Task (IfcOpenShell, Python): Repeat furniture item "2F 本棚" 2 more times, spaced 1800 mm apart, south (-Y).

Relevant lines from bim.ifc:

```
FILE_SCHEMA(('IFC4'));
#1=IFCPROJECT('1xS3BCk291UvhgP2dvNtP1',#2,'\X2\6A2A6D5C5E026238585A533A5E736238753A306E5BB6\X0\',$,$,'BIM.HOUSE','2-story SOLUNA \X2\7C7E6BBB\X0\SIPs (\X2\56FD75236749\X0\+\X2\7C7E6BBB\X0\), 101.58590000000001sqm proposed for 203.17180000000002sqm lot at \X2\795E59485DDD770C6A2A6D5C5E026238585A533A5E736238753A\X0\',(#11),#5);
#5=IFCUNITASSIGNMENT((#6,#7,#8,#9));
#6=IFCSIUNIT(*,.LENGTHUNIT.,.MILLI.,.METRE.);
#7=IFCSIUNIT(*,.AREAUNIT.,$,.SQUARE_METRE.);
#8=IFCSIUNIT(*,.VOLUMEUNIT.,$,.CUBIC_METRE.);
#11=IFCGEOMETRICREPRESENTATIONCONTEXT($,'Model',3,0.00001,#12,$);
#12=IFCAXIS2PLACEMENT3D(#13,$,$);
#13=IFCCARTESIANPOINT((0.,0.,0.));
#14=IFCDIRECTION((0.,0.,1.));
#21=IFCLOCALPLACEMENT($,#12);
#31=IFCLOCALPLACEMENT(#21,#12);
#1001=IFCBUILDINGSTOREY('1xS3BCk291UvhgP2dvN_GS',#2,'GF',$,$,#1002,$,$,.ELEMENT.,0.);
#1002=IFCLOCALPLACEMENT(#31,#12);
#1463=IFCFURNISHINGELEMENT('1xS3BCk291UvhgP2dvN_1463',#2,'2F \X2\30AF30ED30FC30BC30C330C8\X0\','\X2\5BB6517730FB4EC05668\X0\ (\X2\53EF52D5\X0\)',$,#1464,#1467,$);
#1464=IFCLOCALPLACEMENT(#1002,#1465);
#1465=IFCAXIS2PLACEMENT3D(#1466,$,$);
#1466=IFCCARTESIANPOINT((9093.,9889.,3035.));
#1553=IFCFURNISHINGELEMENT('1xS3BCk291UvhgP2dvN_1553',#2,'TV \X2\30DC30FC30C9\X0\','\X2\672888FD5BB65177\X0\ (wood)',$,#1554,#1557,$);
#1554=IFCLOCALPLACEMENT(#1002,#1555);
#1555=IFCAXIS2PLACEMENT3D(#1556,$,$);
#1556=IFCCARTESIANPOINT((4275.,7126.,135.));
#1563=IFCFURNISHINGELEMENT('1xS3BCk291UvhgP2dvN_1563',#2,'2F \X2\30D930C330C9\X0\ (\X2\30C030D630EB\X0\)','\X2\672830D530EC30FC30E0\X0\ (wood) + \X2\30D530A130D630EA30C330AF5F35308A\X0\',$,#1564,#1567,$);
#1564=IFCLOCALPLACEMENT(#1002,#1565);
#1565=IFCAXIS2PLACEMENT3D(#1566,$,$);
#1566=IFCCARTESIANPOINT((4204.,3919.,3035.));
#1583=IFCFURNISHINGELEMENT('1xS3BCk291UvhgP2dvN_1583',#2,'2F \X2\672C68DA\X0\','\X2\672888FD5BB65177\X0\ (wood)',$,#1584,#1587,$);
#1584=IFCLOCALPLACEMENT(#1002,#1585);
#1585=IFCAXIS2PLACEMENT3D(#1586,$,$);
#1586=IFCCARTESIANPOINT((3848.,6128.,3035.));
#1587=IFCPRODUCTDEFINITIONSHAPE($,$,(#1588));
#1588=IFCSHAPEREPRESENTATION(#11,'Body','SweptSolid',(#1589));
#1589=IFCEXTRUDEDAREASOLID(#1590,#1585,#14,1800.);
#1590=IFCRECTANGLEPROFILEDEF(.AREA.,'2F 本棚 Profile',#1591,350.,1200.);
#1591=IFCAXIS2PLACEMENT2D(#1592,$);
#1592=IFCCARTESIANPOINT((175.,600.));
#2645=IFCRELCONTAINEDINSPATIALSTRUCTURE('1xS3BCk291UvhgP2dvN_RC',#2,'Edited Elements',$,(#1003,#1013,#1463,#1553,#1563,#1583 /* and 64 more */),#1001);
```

```python
import numpy as np
import ifcopenshell
import ifcopenshell.api.geometry
import ifcopenshell.api.root
import ifcopenshell.util.element
import ifcopenshell.util.placement

model = ifcopenshell.open("bim.ifc")


def reuse_history(source, copy):
    """copy_class also copies each property set's owner history, people and application; keep the originals."""
    for rel in copy.IsDefinedBy:
        if rel.is_a("IfcRelDefinesByProperties") and (history := rel.RelatingPropertyDefinition.OwnerHistory):
            rel.RelatingPropertyDefinition.OwnerHistory = source.OwnerHistory
            ifcopenshell.util.element.remove_deep2(model, history)


source = model.by_guid("1xS3BCk291UvhgP2dvN_1583")
base = ifcopenshell.util.placement.get_local_placement(source.ObjectPlacement)
step = np.array([0.0, -1.0, 0.0]) * 1800.0

for i in range(1, 3):
    copy = ifcopenshell.api.root.copy_class(model, product=source)
    copy.Representation = ifcopenshell.util.element.copy_deep(
        model, source.Representation, exclude=["IfcGeometricRepresentationContext", "IfcRepresentationMap"]
    )
    reuse_history(source, copy)
    matrix = base.copy()
    matrix[:3, 3] += i * step
    print("added at", matrix[:3, 3].round(3) + 0.0)
    ifcopenshell.api.geometry.edit_object_placement(model, product=copy, matrix=matrix, is_si=False)

model.write("bim-out.ifc")
```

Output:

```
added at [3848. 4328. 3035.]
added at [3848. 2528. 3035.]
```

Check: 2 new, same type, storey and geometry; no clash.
